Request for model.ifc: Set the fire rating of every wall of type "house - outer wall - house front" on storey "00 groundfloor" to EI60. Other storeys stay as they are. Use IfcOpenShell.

First a look at what the model holds.

```python
import ifcopenshell
import ifcopenshell.util.element

model = ifcopenshell.open("model.ifc")
print(model.schema)
storey = next(s for s in model.by_type("IfcBuildingStorey") if s.Name == "00 groundfloor")
walls = [e for e in ifcopenshell.util.element.get_decomposition(storey) if e.is_a("IfcWall")]
seen = {}
for e in walls:
    element_type = ifcopenshell.util.element.get_type(e)
    key = (element_type.Name if element_type != e and element_type else None, ifcopenshell.util.element.get_pset(e, "Pset_WallCommon", "FireRating"))
    seen[key] = seen.get(key, 0) + 1
for (name, value), count in sorted(seen.items(), key=str):
    print(count, "x", name, "|", value)
```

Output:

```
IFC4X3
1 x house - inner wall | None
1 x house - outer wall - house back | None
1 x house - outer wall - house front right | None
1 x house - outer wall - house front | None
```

```python
import ifcopenshell
import ifcopenshell.api.pset
import ifcopenshell.util.element

model = ifcopenshell.open("model.ifc")

storey = next(s for s in model.by_type("IfcBuildingStorey") if s.Name == "00 groundfloor")
walls = [e for e in ifcopenshell.util.element.get_decomposition(storey) if e.is_a("IfcWall")]

count = 0
for e in walls:
    element_type = ifcopenshell.util.element.get_type(e)
    if element_type in (None, e) or element_type.Name != "house - outer wall - house front":
        continue
    # add_pset returns the element's existing set when there is one.
    pset = ifcopenshell.api.pset.add_pset(model, product=e, name="Pset_WallCommon")
    ifcopenshell.api.pset.edit_pset(model, pset=pset, properties={"FireRating": "EI60"})
    count += 1

print(count, "walls updated")

model.write("model_v2.ifc")
```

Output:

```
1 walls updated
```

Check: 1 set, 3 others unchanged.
